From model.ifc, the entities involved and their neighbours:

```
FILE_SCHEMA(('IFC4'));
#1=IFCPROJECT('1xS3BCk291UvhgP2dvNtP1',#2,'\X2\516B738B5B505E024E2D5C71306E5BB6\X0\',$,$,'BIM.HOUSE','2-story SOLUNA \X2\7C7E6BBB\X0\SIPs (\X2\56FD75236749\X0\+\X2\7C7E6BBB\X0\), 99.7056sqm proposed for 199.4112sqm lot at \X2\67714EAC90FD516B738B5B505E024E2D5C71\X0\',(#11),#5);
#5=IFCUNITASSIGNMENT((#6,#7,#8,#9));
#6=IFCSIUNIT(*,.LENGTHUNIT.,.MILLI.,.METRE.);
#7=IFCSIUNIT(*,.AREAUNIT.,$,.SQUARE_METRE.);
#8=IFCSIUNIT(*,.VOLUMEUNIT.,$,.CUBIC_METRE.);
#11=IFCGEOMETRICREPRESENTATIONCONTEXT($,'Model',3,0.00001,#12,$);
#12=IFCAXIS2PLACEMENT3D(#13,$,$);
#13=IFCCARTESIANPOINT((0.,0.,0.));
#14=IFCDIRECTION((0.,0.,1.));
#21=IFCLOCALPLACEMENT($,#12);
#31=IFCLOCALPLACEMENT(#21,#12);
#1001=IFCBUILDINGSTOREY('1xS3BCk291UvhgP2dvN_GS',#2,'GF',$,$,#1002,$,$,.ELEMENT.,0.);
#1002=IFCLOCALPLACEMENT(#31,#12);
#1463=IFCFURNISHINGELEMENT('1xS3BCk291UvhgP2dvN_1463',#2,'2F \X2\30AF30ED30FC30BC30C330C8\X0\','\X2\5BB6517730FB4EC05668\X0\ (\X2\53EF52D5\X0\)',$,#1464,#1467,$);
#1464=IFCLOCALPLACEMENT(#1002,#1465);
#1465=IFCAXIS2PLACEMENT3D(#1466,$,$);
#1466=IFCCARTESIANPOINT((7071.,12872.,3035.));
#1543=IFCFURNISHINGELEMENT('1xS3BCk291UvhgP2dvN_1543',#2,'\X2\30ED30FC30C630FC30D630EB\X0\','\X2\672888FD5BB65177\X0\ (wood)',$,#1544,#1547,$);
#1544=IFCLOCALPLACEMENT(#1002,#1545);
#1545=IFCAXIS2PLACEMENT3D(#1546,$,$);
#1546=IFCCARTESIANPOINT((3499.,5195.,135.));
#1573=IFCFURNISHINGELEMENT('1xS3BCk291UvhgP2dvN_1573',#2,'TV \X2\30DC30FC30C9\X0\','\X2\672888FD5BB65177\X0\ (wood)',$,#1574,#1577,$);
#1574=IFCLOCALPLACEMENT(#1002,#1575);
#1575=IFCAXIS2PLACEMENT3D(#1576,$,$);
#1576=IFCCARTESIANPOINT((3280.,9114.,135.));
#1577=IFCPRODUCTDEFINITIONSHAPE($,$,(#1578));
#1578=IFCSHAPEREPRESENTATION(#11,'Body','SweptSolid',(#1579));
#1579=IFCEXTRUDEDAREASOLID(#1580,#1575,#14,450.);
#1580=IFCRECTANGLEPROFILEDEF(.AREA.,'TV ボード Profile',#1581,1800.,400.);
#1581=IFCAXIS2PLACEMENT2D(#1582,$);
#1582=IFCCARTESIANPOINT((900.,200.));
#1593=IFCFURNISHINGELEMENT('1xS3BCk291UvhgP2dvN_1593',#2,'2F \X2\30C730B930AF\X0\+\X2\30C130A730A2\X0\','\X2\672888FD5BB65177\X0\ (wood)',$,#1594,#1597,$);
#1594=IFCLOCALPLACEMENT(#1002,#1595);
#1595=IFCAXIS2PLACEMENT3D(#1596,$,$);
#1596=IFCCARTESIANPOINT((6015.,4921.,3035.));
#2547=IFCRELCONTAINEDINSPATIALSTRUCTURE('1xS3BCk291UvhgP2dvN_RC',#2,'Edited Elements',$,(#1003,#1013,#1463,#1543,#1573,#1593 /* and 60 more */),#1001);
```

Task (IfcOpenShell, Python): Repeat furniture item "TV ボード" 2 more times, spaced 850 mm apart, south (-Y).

```python
import numpy as np
import ifcopenshell
import ifcopenshell.api.geometry
import ifcopenshell.api.root
import ifcopenshell.util.element
import ifcopenshell.util.placement
import ifcopenshell.util.unit

model = ifcopenshell.open("model.ifc")
unit_scale = ifcopenshell.util.unit.calculate_unit_scale(model)


def reuse_history(source, copy):
    """copy_class also copies each property set's owner history, people and application; keep the originals."""
    for rel in copy.IsDefinedBy:
        if rel.is_a("IfcRelDefinesByProperties") and (history := rel.RelatingPropertyDefinition.OwnerHistory):
            rel.RelatingPropertyDefinition.OwnerHistory = source.OwnerHistory
            ifcopenshell.util.element.remove_deep2(model, history)


source = model.by_id(1573)
base = ifcopenshell.util.placement.get_local_placement(source.ObjectPlacement)
step = np.array([0.0, -1.0, 0.0]) * 0.85 / unit_scale

for i in range(1, 3):
    copy = ifcopenshell.api.root.copy_class(model, product=source)
    copy.Representation = ifcopenshell.util.element.copy_deep(
        model, source.Representation, exclude=["IfcGeometricRepresentationContext", "IfcRepresentationMap"]
    )
    reuse_history(source, copy)
    matrix = base.copy()
    matrix[:3, 3] += i * step
    print("added at", matrix[:3, 3].round(3) + 0.0)
    ifcopenshell.api.geometry.edit_object_placement(model, product=copy, matrix=matrix, is_si=False)

model.write("model_v2.ifc")
```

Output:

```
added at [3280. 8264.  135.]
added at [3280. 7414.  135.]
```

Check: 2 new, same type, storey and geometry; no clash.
